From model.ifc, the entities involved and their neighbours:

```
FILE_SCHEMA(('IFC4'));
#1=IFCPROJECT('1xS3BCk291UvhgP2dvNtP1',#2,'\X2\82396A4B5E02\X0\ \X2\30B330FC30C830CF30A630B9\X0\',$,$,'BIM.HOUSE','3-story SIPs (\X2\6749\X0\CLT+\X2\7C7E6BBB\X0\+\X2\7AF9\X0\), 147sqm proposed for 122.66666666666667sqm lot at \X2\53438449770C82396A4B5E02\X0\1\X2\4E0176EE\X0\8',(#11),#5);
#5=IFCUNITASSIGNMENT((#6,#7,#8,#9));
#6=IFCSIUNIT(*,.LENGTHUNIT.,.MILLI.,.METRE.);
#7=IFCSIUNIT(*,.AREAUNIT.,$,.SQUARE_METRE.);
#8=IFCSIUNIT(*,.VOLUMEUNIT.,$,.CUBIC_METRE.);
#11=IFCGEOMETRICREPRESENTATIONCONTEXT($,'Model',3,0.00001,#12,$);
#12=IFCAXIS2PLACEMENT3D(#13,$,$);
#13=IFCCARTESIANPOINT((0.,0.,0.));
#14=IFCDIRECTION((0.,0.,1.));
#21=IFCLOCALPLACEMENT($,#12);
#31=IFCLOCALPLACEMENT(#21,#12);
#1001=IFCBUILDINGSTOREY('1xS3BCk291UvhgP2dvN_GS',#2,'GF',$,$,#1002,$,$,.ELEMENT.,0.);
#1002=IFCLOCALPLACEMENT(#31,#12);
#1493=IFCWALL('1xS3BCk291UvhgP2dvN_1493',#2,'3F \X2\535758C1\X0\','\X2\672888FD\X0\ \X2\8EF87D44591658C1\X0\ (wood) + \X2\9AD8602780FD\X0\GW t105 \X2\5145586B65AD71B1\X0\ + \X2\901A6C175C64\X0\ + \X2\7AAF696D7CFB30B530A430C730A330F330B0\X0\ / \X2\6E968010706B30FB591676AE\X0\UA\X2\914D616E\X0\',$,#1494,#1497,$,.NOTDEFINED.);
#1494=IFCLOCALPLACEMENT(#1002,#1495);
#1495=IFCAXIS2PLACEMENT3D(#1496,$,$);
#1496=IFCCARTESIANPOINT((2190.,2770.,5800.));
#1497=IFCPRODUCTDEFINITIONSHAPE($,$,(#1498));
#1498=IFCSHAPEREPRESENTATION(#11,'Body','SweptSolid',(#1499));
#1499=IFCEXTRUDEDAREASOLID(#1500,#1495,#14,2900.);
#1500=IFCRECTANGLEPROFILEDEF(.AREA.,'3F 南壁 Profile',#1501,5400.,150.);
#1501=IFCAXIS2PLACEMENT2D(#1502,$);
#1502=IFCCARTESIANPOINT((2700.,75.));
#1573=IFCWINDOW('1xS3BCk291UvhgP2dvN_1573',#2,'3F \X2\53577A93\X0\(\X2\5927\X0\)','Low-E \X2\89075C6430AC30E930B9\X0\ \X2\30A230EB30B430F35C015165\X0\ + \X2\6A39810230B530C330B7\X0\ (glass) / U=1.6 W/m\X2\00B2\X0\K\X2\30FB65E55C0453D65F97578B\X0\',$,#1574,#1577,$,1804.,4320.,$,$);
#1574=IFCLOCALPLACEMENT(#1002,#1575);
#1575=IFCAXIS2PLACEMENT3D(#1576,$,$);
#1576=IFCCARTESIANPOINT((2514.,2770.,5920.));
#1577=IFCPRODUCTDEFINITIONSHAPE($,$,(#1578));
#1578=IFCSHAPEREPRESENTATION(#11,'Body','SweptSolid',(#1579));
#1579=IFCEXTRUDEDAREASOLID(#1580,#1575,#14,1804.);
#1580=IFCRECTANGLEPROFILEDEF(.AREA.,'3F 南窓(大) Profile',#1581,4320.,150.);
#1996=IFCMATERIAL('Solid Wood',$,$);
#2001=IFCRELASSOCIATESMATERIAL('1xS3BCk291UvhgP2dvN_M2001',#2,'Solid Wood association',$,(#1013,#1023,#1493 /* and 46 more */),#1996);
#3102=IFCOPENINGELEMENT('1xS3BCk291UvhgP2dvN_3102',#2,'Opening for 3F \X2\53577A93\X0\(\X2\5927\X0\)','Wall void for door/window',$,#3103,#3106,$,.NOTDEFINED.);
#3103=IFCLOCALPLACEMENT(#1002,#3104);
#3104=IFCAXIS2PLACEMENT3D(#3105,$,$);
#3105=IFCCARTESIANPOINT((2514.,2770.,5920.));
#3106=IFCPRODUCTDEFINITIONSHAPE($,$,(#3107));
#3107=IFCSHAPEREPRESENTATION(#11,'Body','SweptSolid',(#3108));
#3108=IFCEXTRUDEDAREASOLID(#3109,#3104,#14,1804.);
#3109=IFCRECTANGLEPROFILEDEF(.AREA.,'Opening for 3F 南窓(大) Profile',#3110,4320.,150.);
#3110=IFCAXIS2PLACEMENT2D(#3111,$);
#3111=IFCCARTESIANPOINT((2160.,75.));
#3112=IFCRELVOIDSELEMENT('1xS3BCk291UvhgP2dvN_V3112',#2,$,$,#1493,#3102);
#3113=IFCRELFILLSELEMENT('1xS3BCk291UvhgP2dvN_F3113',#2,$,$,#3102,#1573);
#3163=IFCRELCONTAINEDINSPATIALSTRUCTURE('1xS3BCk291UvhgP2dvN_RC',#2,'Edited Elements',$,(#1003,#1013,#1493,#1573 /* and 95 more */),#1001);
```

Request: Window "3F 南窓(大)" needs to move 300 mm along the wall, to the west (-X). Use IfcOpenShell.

```python
import ifcopenshell
import ifcopenshell.api.geometry
import ifcopenshell.util.placement
import ifcopenshell.util.unit

model = ifcopenshell.open("model.ifc")
unit_scale = ifcopenshell.util.unit.calculate_unit_scale(model)

window = model.by_id(1573)
opening = window.FillsVoids[0].RelatingOpeningElement
wall = opening.VoidsElements[0].RelatingBuildingElement

wall_matrix = ifcopenshell.util.placement.get_local_placement(wall.ObjectPlacement)
shift = wall_matrix[:3, 0] * -0.3 / unit_scale
before = ifcopenshell.util.placement.get_local_placement(window.ObjectPlacement)[:3, 3].copy()

# The window is not placed relative to its opening, so move both.
for product in (opening, window):
    matrix = ifcopenshell.util.placement.get_local_placement(product.ObjectPlacement)
    matrix[:3, 3] += shift
    ifcopenshell.api.geometry.edit_object_placement(model, product=product, matrix=matrix, is_si=False)

after = ifcopenshell.util.placement.get_local_placement(window.ObjectPlacement)[:3, 3]
print("window moved by", (after - before).round(3) + 0.0)

model.write("model_rev.ifc")
```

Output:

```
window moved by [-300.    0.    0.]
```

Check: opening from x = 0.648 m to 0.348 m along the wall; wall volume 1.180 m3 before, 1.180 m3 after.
